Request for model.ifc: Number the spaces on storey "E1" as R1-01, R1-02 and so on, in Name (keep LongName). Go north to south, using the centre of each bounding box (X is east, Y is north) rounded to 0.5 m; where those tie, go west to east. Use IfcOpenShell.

First a look at what the model holds.

```python
import ifcopenshell
import ifcopenshell.util.element
import ifcopenshell.util.placement

model = ifcopenshell.open("model.ifc")
print(model.schema)
storey = next(s for s in model.by_type("IfcBuildingStorey") if s.Name == "E1")
spaces = [e for e in ifcopenshell.util.element.get_decomposition(storey) if e.is_a("IfcSpace")]
for e in sorted(spaces, key=lambda e: e.id()):
    origin = ifcopenshell.util.placement.get_local_placement(e.ObjectPlacement)[:3, 3]
    print(e.id(), e.Name, e.LongName, origin.round(2) + 0.0, sep=" | ")
```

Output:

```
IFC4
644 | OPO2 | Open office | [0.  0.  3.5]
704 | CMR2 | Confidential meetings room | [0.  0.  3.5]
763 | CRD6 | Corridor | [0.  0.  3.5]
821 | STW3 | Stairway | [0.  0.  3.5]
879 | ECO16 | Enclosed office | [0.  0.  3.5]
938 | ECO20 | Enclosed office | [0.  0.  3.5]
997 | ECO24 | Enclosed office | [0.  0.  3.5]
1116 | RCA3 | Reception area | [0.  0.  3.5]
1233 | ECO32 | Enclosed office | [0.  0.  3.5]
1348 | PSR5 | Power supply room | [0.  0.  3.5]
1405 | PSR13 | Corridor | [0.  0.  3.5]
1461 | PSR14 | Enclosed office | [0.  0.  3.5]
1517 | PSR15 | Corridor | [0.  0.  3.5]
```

```python
import ifcopenshell
import ifcopenshell.geom
import ifcopenshell.util.element
import ifcopenshell.util.shape

model = ifcopenshell.open("model.ifc")
settings = ifcopenshell.geom.settings()
settings.set("use-world-coords", True)


def centre(element):
    shape = ifcopenshell.geom.create_shape(settings, element)
    return ifcopenshell.util.shape.get_bbox_centroid(shape.geometry)


storey = next(s for s in model.by_type("IfcBuildingStorey") if s.Name == "E1")
spaces = [e for e in ifcopenshell.util.element.get_decomposition(storey) if e.is_a("IfcSpace")]

# Insertion points can sit at a corner or the storey origin, so sort by the geometry (in metres).
centres = {e: centre(e) for e in spaces}
spaces.sort(key=lambda e: (-round(centres[e][1] / 0.5), centres[e][0]))

for i, e in enumerate(spaces, start=1):
    number = f"R1-{i:02d}"
    e.Name = number
    print(e.id(), number)

model.write("model_v2.ifc")
```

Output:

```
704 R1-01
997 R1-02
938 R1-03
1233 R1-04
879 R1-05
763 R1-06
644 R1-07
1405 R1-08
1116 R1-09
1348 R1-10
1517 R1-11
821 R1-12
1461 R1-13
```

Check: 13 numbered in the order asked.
